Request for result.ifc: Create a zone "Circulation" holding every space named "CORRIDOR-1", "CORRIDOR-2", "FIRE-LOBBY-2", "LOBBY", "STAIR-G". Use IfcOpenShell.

First a look at what the model holds.

```python
import ifcopenshell

model = ifcopenshell.open("result.ifc")
print(model.schema)
seen = {}
for space in model.by_type("IfcSpace"):
    seen[space.Name] = seen.get(space.Name, 0) + 1
for name, count in sorted(seen.items(), key=str):
    print(count, "x", name)
print("zones:", [z.Name for z in model.by_type("IfcZone")][:20])
```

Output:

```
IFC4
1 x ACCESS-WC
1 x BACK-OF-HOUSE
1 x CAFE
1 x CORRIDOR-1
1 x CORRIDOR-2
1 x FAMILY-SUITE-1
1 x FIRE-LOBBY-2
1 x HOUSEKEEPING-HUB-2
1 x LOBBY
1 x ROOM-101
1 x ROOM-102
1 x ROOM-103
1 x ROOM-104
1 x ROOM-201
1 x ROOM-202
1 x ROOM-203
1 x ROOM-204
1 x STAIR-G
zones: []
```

```python
import ifcopenshell
import ifcopenshell.api.group
import ifcopenshell.api.root

model = ifcopenshell.open("result.ifc")

names = {"CORRIDOR-1", "CORRIDOR-2", "FIRE-LOBBY-2", "LOBBY", "STAIR-G"}
spaces = [s for s in model.by_type("IfcSpace") if s.Name in names]

zone = ifcopenshell.api.root.create_entity(model, ifc_class="IfcZone", name="Circulation")
ifcopenshell.api.group.assign_group(model, products=spaces, group=zone)
print(len(spaces), "spaces in", zone.Name)

model.write("result-out.ifc")
```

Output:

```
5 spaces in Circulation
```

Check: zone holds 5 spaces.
